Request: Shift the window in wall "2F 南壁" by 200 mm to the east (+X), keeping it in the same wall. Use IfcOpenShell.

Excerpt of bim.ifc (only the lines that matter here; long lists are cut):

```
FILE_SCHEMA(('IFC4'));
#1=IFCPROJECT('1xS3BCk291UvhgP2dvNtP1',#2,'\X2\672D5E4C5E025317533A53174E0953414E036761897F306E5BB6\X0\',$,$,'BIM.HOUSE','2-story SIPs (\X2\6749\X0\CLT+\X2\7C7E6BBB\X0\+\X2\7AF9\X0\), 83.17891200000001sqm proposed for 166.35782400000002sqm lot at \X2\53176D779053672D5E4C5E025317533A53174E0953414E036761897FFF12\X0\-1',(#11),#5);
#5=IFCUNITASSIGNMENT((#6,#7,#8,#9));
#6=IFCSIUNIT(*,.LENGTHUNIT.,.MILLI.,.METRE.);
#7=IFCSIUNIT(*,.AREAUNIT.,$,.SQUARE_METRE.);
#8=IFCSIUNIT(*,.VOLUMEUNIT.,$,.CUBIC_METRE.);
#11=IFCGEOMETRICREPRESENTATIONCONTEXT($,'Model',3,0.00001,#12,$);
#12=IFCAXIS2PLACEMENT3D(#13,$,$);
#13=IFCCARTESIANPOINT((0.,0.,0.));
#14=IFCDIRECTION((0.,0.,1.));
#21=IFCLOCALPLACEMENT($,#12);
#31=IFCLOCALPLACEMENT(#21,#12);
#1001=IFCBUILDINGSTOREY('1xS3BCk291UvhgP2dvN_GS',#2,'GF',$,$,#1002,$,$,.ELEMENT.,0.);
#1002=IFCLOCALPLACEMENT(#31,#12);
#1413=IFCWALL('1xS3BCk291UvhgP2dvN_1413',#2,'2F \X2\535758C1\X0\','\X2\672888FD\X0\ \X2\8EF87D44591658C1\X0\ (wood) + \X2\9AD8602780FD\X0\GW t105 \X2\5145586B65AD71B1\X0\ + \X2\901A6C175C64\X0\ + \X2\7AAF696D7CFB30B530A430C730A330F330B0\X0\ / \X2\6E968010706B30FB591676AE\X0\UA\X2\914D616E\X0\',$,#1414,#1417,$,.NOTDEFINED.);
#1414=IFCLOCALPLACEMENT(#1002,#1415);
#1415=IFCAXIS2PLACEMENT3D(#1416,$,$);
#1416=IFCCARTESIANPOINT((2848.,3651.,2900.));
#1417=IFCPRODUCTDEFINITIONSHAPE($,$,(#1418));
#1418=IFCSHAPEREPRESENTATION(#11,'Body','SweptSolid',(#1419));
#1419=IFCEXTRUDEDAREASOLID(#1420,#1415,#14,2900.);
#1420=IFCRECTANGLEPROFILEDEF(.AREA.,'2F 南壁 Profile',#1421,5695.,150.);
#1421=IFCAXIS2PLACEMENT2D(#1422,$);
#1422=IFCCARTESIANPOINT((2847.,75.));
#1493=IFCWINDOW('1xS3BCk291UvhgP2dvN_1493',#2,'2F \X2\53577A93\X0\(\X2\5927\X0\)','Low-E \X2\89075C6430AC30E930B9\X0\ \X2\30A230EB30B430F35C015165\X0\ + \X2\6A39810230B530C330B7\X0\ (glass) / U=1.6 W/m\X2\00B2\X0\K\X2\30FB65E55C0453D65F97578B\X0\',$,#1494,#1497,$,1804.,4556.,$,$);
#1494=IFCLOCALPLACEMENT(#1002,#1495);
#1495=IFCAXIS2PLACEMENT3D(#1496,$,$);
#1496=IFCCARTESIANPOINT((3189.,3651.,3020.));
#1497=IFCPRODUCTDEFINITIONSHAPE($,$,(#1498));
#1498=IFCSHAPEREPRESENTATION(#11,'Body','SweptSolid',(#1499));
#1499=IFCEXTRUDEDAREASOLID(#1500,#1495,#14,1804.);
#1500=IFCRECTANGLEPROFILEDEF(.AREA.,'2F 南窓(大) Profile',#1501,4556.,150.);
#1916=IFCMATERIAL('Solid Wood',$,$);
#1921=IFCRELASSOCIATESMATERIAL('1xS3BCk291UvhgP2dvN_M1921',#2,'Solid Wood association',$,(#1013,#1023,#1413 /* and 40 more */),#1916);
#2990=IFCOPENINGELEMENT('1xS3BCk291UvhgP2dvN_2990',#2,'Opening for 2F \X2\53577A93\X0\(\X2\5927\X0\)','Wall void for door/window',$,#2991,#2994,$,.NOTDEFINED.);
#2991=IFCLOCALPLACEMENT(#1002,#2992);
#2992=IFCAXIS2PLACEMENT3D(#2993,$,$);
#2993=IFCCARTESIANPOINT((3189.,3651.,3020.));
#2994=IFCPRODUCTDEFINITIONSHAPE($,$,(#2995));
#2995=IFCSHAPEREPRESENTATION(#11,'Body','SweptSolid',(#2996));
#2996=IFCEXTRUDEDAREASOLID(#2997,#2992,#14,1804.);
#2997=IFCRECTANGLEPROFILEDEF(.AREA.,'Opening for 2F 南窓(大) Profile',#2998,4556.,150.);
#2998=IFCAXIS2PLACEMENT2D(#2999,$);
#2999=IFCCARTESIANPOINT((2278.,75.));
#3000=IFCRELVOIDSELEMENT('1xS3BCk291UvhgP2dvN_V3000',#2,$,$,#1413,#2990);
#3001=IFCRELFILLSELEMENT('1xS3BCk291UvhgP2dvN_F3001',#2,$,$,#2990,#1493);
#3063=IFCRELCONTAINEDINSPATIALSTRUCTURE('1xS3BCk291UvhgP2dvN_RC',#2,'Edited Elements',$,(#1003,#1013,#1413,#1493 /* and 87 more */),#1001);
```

```python
import ifcopenshell
import ifcopenshell.api.geometry
import ifcopenshell.util.placement

model = ifcopenshell.open("bim.ifc")

window = model.by_guid("1xS3BCk291UvhgP2dvN_1493")
opening = window.FillsVoids[0].RelatingOpeningElement
wall = opening.VoidsElements[0].RelatingBuildingElement

wall_matrix = ifcopenshell.util.placement.get_local_placement(wall.ObjectPlacement)
shift = wall_matrix[:3, 0] * 200.0
before = ifcopenshell.util.placement.get_local_placement(window.ObjectPlacement)[:3, 3].copy()

# The window is not placed relative to its opening, so move both.
for product in (opening, window):
    matrix = ifcopenshell.util.placement.get_local_placement(product.ObjectPlacement)
    matrix[:3, 3] += shift
    ifcopenshell.api.geometry.edit_object_placement(model, product=product, matrix=matrix, is_si=False)

after = ifcopenshell.util.placement.get_local_placement(window.ObjectPlacement)[:3, 3]
print("window moved by", (after - before).round(3) + 0.0)

model.write("bim-out.ifc")
```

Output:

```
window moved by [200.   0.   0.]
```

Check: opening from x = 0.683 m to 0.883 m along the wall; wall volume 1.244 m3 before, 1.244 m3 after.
